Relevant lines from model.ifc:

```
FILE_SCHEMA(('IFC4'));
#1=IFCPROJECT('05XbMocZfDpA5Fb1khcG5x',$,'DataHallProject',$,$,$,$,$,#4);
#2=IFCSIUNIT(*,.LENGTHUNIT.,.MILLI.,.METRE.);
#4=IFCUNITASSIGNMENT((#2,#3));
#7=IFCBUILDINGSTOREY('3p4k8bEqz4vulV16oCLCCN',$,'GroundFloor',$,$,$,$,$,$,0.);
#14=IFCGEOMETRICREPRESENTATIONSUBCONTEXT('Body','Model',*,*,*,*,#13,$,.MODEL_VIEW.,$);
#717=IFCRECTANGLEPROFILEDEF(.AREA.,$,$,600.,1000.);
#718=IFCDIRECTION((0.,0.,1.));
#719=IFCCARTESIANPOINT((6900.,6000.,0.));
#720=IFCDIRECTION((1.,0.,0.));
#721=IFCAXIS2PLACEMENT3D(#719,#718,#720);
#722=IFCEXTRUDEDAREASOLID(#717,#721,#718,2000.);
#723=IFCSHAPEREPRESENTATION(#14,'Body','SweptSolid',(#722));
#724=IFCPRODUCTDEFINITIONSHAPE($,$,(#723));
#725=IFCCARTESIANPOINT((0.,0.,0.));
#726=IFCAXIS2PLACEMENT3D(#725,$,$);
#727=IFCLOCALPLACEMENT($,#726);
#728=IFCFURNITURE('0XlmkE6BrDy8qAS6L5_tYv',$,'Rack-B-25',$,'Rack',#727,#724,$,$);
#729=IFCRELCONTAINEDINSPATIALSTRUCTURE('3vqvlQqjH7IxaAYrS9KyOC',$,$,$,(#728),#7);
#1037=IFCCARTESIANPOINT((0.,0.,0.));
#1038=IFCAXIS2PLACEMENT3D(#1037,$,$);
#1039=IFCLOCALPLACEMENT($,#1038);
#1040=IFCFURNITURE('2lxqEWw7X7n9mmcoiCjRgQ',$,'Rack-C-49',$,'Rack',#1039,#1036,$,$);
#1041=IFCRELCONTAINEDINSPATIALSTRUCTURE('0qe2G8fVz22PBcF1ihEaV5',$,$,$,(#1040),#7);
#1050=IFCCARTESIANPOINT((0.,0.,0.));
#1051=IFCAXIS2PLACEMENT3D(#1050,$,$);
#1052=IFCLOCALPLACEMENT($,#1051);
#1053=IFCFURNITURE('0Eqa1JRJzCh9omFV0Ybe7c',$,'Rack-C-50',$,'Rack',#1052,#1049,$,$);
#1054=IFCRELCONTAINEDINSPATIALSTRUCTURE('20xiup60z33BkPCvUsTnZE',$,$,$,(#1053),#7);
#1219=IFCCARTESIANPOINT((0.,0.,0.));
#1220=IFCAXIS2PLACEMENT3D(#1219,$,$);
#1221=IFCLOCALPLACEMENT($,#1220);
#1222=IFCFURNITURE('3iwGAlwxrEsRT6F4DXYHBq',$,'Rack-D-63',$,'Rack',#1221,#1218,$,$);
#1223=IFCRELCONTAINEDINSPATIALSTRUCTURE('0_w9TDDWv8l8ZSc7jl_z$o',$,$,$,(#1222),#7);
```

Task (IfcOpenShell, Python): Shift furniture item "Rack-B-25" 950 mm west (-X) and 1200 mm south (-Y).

```python
import ifcopenshell
import ifcopenshell.api.geometry
import ifcopenshell.util.placement
import ifcopenshell.util.unit

model = ifcopenshell.open("model.ifc")
unit_scale = ifcopenshell.util.unit.calculate_unit_scale(model)

item = model.by_guid("0XlmkE6BrDy8qAS6L5_tYv")
matrix = ifcopenshell.util.placement.get_local_placement(item.ObjectPlacement)
matrix[0, 3] -= 0.95 / unit_scale
matrix[1, 3] -= 1.2 / unit_scale
ifcopenshell.api.geometry.edit_object_placement(model, product=item, matrix=matrix, is_si=False)

print(ifcopenshell.util.placement.get_local_placement(item.ObjectPlacement).round(3) + 0.0)

model.write("model_v2.ifc")
```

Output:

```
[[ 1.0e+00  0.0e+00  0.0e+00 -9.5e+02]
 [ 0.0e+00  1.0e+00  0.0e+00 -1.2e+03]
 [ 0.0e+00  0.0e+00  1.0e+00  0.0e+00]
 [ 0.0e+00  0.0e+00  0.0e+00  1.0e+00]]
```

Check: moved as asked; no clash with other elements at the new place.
